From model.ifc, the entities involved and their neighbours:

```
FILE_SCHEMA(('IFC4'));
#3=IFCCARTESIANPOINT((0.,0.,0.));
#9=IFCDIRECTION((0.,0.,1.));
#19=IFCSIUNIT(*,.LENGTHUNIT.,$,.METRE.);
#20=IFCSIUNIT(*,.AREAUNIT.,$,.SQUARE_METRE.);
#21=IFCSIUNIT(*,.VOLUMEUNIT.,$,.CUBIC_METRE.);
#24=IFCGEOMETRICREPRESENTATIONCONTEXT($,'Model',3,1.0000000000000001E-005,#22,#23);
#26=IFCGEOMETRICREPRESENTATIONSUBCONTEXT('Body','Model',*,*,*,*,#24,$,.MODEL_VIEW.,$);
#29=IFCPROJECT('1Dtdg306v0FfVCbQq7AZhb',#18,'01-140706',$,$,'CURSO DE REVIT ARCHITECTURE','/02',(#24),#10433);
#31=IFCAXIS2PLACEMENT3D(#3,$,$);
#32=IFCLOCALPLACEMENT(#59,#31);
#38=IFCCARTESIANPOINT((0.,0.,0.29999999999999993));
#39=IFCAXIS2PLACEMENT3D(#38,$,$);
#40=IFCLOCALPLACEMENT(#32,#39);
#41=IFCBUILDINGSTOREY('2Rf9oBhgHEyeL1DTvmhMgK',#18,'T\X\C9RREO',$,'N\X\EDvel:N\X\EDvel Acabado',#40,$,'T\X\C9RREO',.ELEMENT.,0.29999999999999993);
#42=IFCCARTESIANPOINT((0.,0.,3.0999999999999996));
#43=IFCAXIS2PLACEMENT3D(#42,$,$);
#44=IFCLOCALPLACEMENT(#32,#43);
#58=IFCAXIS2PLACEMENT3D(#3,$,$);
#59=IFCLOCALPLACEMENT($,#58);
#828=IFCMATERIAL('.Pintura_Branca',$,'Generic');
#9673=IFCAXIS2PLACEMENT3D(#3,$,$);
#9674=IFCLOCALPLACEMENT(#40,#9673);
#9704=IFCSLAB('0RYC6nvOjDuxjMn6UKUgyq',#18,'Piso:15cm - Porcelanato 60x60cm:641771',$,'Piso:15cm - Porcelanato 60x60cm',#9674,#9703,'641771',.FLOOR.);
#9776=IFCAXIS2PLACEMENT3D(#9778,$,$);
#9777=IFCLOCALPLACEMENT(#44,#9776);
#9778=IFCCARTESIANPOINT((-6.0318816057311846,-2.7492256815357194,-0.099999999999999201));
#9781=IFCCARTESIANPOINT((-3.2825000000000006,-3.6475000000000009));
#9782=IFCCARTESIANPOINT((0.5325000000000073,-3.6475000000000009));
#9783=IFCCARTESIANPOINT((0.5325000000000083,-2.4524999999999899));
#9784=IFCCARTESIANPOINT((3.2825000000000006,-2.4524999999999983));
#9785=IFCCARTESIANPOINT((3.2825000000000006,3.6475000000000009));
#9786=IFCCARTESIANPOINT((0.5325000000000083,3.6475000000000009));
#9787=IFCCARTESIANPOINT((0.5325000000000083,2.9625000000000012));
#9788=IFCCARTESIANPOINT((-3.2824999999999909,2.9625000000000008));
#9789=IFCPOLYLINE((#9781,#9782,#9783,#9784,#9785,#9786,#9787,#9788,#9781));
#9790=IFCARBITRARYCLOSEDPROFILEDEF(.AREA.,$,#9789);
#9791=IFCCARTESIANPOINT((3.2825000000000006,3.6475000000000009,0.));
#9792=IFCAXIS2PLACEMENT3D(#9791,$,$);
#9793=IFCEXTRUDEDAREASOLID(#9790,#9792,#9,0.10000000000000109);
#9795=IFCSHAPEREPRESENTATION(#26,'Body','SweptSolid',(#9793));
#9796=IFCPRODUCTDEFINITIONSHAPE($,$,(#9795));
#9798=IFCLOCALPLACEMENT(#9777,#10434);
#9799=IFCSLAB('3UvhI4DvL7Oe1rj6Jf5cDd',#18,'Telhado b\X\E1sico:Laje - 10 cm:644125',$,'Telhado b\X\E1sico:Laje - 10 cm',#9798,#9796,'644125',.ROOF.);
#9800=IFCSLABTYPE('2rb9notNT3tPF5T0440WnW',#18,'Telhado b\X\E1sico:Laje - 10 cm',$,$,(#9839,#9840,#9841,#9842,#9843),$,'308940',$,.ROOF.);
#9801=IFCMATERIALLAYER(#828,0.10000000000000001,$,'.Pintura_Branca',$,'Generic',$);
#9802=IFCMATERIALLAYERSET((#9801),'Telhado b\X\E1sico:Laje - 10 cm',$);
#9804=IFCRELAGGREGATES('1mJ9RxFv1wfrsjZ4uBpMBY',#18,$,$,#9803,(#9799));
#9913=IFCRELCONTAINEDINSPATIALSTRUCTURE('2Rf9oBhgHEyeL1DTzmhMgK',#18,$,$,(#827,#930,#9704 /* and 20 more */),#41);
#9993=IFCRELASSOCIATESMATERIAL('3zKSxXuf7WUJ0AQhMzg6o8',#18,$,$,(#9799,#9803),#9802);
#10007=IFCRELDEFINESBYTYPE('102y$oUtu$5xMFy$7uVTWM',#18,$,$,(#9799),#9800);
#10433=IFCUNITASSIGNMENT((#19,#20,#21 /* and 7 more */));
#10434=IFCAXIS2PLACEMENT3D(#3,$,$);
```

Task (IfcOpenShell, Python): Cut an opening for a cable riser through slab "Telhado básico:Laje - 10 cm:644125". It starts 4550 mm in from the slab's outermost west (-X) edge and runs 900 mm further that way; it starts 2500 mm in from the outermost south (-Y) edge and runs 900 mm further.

```python
import numpy as np
import ifcopenshell
import ifcopenshell.api.feature
import ifcopenshell.api.geometry
import ifcopenshell.api.root
import ifcopenshell.geom
import ifcopenshell.util.placement
import ifcopenshell.util.representation
import ifcopenshell.util.shape
import ifcopenshell.util.unit

model = ifcopenshell.open("model.ifc")
unit_scale = ifcopenshell.util.unit.calculate_unit_scale(model)
settings = ifcopenshell.geom.settings()


def volume(element):
    """Net volume in cubic metres, openings subtracted."""
    shape = ifcopenshell.geom.create_shape(settings, element)
    return ifcopenshell.util.shape.get_volume(shape.geometry)


slab = model.by_id(9799)
before = volume(slab)

# Extent in the slab's own axes, in metres. The edges named are its -X and -Y sides.
slab_shape = ifcopenshell.geom.create_shape(settings, slab)
vertices = ifcopenshell.util.shape.get_vertices(slab_shape.geometry)
x_min, y_min, bottom = vertices.min(axis=0)
top = vertices[:, 2].max()

opening = ifcopenshell.api.root.create_entity(model, ifc_class="IfcOpeningElement", name="Cable riser opening", predefined_type="OPENING")
context = ifcopenshell.util.representation.get_context(model, "Model", "Body", "MODEL_VIEW")
width, depth = 0.9, 0.9
outline = [(0.0, 0.0), (width, 0.0), (width, depth), (0.0, depth), (0.0, 0.0)]
# Overshoot both faces by 50 mm so the cut is clean.
shape = ifcopenshell.api.geometry.add_slab_representation(
    model, context=context, depth=top - bottom + 0.1, polyline=outline
)
ifcopenshell.api.geometry.assign_representation(model, product=opening, representation=shape)

matrix = ifcopenshell.util.placement.get_local_placement(slab.ObjectPlacement)
matrix[:, 3] = matrix @ np.append(np.array([x_min + 4.55, y_min + 2.5, bottom - 0.05]) / unit_scale, 1.0)
ifcopenshell.api.geometry.edit_object_placement(model, product=opening, matrix=matrix, is_si=False)
ifcopenshell.api.feature.add_feature(model, feature=opening, element=slab)

after = volume(slab)

print(f"slab volume {before:.3f} -> {after:.3f} m3")

model.write("model-out.ifc")
```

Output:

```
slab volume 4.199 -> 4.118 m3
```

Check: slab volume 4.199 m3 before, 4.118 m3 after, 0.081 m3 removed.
